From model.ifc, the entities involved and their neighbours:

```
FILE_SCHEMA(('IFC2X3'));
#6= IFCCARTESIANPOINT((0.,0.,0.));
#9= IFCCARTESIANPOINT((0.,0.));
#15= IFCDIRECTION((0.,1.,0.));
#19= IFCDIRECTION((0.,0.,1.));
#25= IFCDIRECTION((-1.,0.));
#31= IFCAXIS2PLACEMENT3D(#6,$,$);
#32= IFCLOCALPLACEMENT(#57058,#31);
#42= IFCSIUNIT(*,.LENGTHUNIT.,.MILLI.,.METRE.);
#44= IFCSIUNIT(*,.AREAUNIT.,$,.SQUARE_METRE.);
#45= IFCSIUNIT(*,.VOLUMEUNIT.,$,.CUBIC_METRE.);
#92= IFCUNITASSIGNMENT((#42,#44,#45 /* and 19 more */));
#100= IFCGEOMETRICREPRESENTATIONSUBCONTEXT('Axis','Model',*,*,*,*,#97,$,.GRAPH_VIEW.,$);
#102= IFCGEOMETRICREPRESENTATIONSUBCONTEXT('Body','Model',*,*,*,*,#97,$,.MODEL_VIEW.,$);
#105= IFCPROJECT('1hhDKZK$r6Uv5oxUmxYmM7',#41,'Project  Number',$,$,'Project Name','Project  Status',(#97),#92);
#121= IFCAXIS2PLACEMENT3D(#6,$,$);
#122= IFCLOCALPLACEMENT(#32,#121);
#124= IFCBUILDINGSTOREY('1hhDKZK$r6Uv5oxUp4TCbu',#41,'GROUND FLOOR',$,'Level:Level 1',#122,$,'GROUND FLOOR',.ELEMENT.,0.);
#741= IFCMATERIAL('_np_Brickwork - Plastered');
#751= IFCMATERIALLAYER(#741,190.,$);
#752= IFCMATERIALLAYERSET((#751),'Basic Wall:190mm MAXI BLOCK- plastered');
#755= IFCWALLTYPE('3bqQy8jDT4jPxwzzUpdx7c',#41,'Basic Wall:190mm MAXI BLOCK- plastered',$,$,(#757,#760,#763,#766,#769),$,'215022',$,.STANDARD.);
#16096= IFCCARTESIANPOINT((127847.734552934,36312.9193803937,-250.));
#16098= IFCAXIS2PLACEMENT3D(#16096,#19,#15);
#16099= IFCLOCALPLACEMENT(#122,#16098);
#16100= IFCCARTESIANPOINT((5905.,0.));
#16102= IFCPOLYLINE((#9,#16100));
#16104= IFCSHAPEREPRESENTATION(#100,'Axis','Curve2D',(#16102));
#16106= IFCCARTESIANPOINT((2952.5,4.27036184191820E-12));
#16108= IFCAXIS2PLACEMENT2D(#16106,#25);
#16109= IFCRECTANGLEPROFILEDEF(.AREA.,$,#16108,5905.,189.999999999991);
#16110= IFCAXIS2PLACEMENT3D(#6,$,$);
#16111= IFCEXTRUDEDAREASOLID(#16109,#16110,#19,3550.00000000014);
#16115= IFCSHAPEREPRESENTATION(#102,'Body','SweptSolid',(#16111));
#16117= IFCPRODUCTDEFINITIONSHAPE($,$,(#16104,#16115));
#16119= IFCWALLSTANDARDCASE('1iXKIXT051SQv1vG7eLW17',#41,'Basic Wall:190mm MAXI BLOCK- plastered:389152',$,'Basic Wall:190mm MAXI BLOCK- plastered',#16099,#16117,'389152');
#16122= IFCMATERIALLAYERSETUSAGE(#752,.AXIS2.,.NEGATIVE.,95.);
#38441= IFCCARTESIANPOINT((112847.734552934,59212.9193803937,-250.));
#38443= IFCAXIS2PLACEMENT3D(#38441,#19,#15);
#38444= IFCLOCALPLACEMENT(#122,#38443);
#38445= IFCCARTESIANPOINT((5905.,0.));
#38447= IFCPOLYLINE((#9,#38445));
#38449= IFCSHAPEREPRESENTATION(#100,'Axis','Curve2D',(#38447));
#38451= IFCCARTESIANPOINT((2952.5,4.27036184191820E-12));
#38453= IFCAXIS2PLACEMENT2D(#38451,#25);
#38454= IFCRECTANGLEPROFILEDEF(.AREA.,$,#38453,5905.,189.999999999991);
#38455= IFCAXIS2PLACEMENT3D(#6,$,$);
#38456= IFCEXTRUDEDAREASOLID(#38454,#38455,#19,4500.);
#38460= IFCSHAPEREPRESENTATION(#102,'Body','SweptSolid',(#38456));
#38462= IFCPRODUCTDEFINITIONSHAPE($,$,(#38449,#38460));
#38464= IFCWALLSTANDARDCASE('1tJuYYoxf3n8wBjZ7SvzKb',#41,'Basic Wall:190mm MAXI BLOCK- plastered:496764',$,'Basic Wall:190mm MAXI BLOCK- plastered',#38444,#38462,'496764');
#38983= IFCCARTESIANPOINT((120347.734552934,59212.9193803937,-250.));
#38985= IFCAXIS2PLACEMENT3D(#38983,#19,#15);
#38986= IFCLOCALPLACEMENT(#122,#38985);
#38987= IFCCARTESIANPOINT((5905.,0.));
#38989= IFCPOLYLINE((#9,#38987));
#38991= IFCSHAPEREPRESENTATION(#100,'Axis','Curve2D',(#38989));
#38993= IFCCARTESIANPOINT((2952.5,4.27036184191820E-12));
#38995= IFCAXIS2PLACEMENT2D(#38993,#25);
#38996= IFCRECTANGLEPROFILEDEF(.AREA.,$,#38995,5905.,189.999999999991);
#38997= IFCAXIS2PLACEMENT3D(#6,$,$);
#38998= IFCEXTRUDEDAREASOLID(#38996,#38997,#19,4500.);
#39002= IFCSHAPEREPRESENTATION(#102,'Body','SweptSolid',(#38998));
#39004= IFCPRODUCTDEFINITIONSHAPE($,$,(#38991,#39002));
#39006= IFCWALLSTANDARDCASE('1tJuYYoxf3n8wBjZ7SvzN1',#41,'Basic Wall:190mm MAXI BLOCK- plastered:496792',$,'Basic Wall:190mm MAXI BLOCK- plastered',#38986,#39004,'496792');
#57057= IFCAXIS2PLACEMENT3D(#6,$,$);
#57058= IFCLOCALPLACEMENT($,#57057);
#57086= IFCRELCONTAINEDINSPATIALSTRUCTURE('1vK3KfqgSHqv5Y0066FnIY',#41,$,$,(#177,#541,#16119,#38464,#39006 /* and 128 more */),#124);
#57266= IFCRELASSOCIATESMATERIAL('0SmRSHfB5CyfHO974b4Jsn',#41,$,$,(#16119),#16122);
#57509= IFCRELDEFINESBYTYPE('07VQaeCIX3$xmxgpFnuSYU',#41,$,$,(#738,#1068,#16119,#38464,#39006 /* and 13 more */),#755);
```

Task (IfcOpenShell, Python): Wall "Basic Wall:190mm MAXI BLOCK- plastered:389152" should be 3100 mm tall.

```python
import ifcopenshell
import ifcopenshell.geom
import ifcopenshell.util.representation
import ifcopenshell.util.shape
import ifcopenshell.util.unit

model = ifcopenshell.open("model.ifc")
unit_scale = ifcopenshell.util.unit.calculate_unit_scale(model)
settings = ifcopenshell.geom.settings()


def volume(element):
    """Net volume in cubic metres, openings subtracted."""
    shape = ifcopenshell.geom.create_shape(settings, element)
    return ifcopenshell.util.shape.get_volume(shape.geometry)


wall = model.by_guid("1iXKIXT051SQv1vG7eLW17")
before = volume(wall)

body = ifcopenshell.util.representation.get_representation(wall, "Model", "Body")
solid = body.Items[0]
old_height = solid.Depth
solid.Depth = 3.1 / unit_scale
after = volume(wall)

print(f"height {old_height:g} -> {solid.Depth:g}, volume {before:.3f} -> {after:.3f} m3")

model.write("model_rev.ifc")
```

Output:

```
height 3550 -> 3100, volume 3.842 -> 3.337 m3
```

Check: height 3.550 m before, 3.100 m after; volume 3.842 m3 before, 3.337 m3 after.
